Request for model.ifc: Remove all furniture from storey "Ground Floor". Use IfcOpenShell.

First a look at what the model holds.

```python
import ifcopenshell
import ifcopenshell.util.element

model = ifcopenshell.open("model.ifc")
print(model.schema)
storey = next(s for s in model.by_type("IfcBuildingStorey") if s.Name == "Ground Floor")
furniture = [e for e in ifcopenshell.util.element.get_decomposition(storey) if e.is_a("IfcFurnishingElement")]
seen = {}
for e in furniture:
    element_type = ifcopenshell.util.element.get_type(e)
    name = element_type.Name if element_type not in (None, e) else None
    seen[name] = seen.get(name, 0) + 1
for name, count in sorted(seen.items(), key=str):
    print(count, "x", name)
```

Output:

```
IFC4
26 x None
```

```python
import ifcopenshell
import ifcopenshell.api.root
import ifcopenshell.util.element

model = ifcopenshell.open("model.ifc")

storey = next(s for s in model.by_type("IfcBuildingStorey") if s.Name == "Ground Floor")
furniture = [e for e in ifcopenshell.util.element.get_decomposition(storey) if e.is_a("IfcFurnishingElement")]

for e in furniture:
    ifcopenshell.api.root.remove_product(model, product=e)
print(len(furniture), "removed")

model.write("model-out.ifc")
```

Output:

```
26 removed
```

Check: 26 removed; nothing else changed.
